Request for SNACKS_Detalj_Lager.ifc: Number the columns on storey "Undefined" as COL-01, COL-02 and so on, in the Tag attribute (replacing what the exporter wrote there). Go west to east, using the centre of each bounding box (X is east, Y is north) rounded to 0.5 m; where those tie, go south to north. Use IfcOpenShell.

First a look at what the model holds.

```python
import ifcopenshell
import ifcopenshell.util.element
import ifcopenshell.util.placement

model = ifcopenshell.open("SNACKS_Detalj_Lager.ifc")
print(model.schema)
storey = next(s for s in model.by_type("IfcBuildingStorey") if s.Name == "Undefined")
columns = [e for e in ifcopenshell.util.element.get_decomposition(storey) if e.is_a("IfcColumn")]
for e in sorted(columns, key=lambda e: e.id()):
    origin = ifcopenshell.util.placement.get_local_placement(e.ObjectPlacement)[:3, 3]
    print(e.id(), e.Tag, e.Name, origin.round(2) + 0.0, sep=" | ")
```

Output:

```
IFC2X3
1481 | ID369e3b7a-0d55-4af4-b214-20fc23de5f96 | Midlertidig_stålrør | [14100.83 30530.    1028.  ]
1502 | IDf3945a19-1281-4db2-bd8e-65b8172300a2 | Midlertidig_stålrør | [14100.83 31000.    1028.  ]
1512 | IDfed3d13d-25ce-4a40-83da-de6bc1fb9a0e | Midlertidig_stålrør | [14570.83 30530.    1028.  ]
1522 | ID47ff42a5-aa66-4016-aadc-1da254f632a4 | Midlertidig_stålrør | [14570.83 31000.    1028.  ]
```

```python
import ifcopenshell
import ifcopenshell.geom
import ifcopenshell.util.element
import ifcopenshell.util.shape

model = ifcopenshell.open("SNACKS_Detalj_Lager.ifc")
settings = ifcopenshell.geom.settings()
settings.set("use-world-coords", True)


def centre(element):
    shape = ifcopenshell.geom.create_shape(settings, element)
    return ifcopenshell.util.shape.get_bbox_centroid(shape.geometry)


storey = next(s for s in model.by_type("IfcBuildingStorey") if s.Name == "Undefined")
columns = [e for e in ifcopenshell.util.element.get_decomposition(storey) if e.is_a("IfcColumn")]

# Insertion points can sit at a corner or the storey origin, so sort by the geometry (in metres).
centres = {e: centre(e) for e in columns}
columns.sort(key=lambda e: (round(centres[e][0] / 0.5), centres[e][1]))

for i, e in enumerate(columns, start=1):
    number = f"COL-{i:02d}"
    e.Tag = number
    print(e.id(), number)

model.write("SNACKS_Detalj_Lager_edited.ifc")
```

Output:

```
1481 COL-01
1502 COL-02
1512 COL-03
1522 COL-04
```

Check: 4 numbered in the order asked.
